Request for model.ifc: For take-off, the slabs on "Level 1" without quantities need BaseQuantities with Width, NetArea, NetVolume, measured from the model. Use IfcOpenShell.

First a look at what the model holds.

```python
import ifcopenshell
import ifcopenshell.util.element
import ifcopenshell.util.unit

model = ifcopenshell.open("model.ifc")
print(model.schema)
for unit_type in ("LENGTHUNIT", "AREAUNIT", "VOLUMEUNIT"):
    print(unit_type, ifcopenshell.util.unit.calculate_unit_scale(model, unit_type))
storey = next(s for s in model.by_type("IfcBuildingStorey") if s.Name == "Level 1")
slabs = [e for e in ifcopenshell.util.element.get_decomposition(storey) if e.is_a("IfcSlab")]
for e in sorted(slabs, key=lambda e: e.id()):
    print(e.id(), e.is_a(), e.Name, list(ifcopenshell.util.element.get_psets(e, qtos_only=True)), sep=" | ")
```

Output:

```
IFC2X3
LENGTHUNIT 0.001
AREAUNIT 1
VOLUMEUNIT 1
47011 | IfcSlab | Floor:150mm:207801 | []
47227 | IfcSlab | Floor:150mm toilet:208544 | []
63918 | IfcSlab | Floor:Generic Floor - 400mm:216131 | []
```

```python
import ifcopenshell
import ifcopenshell.api.pset
import ifcopenshell.geom
import ifcopenshell.util.element
import ifcopenshell.util.shape
import ifcopenshell.util.unit

model = ifcopenshell.open("model.ifc")
unit_scale = ifcopenshell.util.unit.calculate_unit_scale(model)
area_scale = ifcopenshell.util.unit.calculate_unit_scale(model, "AREAUNIT")
volume_scale = ifcopenshell.util.unit.calculate_unit_scale(model, "VOLUMEUNIT")
settings = ifcopenshell.geom.settings()

storey = next(s for s in model.by_type("IfcBuildingStorey") if s.Name == "Level 1")
slabs = [e for e in ifcopenshell.util.element.get_decomposition(storey) if e.is_a("IfcSlab")]

for e in sorted(slabs, key=lambda e: e.id()):
    if ifcopenshell.util.element.get_psets(e, qtos_only=True, should_inherit=False):
        continue
    # Geometry comes back in metres, in the element's own axes.
    shape = ifcopenshell.geom.create_shape(settings, e)
    values = {
        "Width": ifcopenshell.util.shape.get_z(shape.geometry) / unit_scale,
        "NetArea": ifcopenshell.util.shape.get_footprint_area(shape.geometry) / area_scale,
        "NetVolume": ifcopenshell.util.shape.get_volume(shape.geometry) / volume_scale,
    }
    qto = ifcopenshell.api.pset.add_qto(model, product=e, name="BaseQuantities")
    ifcopenshell.api.pset.edit_qto(model, qto=qto, properties=values)
    print(e.id(), {k: round(v, 3) for k, v in values.items()})

model.write("model_v2.ifc")
```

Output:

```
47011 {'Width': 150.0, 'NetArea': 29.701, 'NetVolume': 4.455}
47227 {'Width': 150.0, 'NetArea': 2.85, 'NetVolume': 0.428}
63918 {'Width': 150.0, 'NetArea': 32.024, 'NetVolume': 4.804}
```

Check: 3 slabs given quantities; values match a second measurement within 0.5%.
